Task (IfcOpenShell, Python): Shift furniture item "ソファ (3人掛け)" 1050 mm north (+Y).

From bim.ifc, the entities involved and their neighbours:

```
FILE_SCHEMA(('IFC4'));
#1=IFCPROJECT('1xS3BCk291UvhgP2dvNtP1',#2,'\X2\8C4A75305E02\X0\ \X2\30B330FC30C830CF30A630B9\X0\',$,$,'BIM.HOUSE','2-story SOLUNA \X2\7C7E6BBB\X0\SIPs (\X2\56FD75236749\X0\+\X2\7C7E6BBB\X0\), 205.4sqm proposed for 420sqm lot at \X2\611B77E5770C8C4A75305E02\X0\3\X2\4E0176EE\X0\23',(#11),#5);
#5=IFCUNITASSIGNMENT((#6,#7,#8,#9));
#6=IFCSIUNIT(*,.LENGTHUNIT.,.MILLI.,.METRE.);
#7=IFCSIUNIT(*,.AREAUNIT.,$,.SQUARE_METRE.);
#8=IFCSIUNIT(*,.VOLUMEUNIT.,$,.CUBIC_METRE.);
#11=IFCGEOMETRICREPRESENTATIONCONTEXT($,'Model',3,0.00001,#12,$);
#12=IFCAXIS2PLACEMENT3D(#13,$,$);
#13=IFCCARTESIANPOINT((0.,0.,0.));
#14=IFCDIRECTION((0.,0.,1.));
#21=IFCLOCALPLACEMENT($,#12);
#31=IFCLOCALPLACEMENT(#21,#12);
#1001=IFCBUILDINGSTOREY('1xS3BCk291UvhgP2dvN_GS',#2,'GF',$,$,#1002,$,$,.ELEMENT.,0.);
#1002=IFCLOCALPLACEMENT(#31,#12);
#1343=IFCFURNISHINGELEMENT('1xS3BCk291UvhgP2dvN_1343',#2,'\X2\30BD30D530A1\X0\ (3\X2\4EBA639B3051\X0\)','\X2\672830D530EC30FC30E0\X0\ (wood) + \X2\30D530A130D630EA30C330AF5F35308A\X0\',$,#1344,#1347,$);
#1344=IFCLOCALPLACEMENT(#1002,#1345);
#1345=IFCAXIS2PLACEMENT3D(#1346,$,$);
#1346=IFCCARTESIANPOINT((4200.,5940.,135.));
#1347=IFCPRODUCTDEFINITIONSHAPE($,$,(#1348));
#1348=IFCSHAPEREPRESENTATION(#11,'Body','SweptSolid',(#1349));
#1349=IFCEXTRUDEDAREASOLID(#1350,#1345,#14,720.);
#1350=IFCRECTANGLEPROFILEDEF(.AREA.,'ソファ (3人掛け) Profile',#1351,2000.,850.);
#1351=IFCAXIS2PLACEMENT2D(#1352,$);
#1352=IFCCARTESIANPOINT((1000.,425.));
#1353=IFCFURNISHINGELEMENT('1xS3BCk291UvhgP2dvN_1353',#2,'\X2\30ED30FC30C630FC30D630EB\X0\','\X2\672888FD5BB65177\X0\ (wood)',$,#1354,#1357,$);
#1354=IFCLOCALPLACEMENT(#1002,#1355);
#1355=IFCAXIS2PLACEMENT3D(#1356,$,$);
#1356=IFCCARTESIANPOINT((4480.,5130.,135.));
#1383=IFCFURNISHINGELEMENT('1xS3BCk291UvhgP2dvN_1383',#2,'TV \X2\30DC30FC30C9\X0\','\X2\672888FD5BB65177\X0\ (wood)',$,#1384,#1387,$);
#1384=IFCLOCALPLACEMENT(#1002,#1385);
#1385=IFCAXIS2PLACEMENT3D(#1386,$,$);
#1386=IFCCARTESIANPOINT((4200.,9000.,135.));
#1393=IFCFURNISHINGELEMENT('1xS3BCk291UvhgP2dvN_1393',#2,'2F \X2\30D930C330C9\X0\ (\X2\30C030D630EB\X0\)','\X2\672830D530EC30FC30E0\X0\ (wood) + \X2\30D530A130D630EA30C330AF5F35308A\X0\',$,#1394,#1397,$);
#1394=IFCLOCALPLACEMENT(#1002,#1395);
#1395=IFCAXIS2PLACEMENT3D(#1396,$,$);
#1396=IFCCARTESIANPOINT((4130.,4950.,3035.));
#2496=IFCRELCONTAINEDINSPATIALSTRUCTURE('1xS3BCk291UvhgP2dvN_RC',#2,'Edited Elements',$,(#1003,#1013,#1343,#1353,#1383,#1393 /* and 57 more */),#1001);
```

```python
import ifcopenshell
import ifcopenshell.api.geometry
import ifcopenshell.util.placement
import ifcopenshell.util.unit

model = ifcopenshell.open("bim.ifc")
unit_scale = ifcopenshell.util.unit.calculate_unit_scale(model)

item = model.by_guid("1xS3BCk291UvhgP2dvN_1343")
matrix = ifcopenshell.util.placement.get_local_placement(item.ObjectPlacement)
matrix[1, 3] += 1.05 / unit_scale
ifcopenshell.api.geometry.edit_object_placement(model, product=item, matrix=matrix, is_si=False)

print(ifcopenshell.util.placement.get_local_placement(item.ObjectPlacement).round(3) + 0.0)

model.write("bim_updated.ifc")
```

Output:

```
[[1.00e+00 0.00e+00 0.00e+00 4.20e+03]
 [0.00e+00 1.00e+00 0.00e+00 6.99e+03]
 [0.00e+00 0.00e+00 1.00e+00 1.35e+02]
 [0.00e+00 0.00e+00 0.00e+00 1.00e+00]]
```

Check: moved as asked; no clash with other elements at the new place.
